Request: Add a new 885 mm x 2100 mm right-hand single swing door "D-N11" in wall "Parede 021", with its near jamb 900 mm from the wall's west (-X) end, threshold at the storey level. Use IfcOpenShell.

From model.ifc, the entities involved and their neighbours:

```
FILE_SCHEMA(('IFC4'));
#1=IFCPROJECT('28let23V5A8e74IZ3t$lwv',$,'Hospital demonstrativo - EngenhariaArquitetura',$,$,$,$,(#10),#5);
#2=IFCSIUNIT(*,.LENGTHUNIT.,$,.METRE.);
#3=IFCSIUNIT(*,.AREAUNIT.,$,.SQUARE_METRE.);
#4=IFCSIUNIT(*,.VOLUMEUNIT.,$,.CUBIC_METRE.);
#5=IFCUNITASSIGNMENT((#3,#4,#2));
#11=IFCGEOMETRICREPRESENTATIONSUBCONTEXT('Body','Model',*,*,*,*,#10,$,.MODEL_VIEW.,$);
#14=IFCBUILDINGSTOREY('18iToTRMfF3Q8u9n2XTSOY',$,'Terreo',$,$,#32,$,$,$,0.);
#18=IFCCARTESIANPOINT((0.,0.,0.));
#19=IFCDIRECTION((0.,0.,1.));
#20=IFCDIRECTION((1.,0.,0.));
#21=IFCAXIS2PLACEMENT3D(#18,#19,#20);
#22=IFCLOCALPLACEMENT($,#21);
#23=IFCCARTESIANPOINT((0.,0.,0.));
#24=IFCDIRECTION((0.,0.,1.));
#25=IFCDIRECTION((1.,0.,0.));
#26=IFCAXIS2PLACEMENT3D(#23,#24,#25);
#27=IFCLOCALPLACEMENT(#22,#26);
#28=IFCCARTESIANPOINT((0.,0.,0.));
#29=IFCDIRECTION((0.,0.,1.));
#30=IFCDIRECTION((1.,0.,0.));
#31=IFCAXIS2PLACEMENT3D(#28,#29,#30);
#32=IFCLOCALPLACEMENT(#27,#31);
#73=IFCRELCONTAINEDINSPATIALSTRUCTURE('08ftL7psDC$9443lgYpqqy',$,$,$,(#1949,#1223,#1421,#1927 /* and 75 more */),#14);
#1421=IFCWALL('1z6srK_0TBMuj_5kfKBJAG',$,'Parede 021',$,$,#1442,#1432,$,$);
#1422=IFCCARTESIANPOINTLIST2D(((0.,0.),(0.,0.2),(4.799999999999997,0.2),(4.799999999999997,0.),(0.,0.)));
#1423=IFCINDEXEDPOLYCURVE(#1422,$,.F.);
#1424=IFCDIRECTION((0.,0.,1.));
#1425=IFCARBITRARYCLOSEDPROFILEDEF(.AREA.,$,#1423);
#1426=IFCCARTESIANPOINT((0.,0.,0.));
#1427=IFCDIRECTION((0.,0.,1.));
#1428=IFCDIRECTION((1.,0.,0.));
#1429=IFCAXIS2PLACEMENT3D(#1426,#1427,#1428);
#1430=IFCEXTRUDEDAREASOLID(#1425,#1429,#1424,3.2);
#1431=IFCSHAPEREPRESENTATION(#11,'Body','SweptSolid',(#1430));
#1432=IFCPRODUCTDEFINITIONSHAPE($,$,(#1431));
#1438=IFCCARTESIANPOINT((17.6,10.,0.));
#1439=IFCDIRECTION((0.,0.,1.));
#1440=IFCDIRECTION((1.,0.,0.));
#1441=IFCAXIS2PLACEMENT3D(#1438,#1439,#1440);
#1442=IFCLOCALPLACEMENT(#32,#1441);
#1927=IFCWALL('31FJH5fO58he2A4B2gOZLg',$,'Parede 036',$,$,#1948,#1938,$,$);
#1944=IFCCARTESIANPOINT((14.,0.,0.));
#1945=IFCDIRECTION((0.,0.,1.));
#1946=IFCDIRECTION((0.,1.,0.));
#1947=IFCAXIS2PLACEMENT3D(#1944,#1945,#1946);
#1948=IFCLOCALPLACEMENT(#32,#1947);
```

```python
import numpy as np
import ifcopenshell
import ifcopenshell.api.feature
import ifcopenshell.api.geometry
import ifcopenshell.api.root
import ifcopenshell.api.spatial
import ifcopenshell.geom
import ifcopenshell.util.element
import ifcopenshell.util.placement
import ifcopenshell.util.representation
import ifcopenshell.util.shape
import ifcopenshell.util.unit

model = ifcopenshell.open("model.ifc")
unit_scale = ifcopenshell.util.unit.calculate_unit_scale(model)
settings = ifcopenshell.geom.settings()


def volume(element):
    """Net volume in cubic metres, openings subtracted."""
    shape = ifcopenshell.geom.create_shape(settings, element)
    return ifcopenshell.util.shape.get_volume(shape.geometry)


wall = model.by_guid("1z6srK_0TBMuj_5kfKBJAG")
storey = ifcopenshell.util.element.get_container(wall, ifc_class="IfcBuildingStorey")
context = ifcopenshell.util.representation.get_context(model, "Model", "Body", "MODEL_VIEW")
before = volume(wall)

width, height, from_end, sill = 0.885, 2.1, 0.9, 0.0  # metres

# The wall runs along its own X axis, and the end named is its -X end.
wall_shape = ifcopenshell.geom.create_shape(settings, wall)
x, y, z = ifcopenshell.util.shape.get_vertices(wall_shape.geometry).T
start = x.min() + from_end
face, thickness = float(y.min()), float(y.max() - y.min())
wall_matrix = ifcopenshell.util.placement.get_local_placement(wall.ObjectPlacement)
level = ifcopenshell.util.placement.get_local_placement(storey.ObjectPlacement)[2, 3]


def in_wall(x, y):
    """Placement at x, y metres in the wall's axes, at sill height."""
    matrix = wall_matrix.copy()
    matrix[:, 3] = wall_matrix @ np.array([x / unit_scale, y / unit_scale, 0.0, 1.0])
    matrix[2, 3] = level + sill / unit_scale
    return matrix


# Opening: a box that overshoots both wall faces by 50 mm.
opening = ifcopenshell.api.root.create_entity(model, ifc_class="IfcOpeningElement", predefined_type="OPENING")
box = ifcopenshell.api.geometry.add_wall_representation(
    model, context=context, length=width, height=height, thickness=thickness + 0.1
)
ifcopenshell.api.geometry.assign_representation(model, product=opening, representation=box)
ifcopenshell.api.geometry.edit_object_placement(model, product=opening, matrix=in_wall(start, face - 0.05), is_si=False)
ifcopenshell.api.feature.add_feature(model, feature=opening, element=wall)

door = ifcopenshell.api.root.create_entity(model, ifc_class="IfcDoor", name="D-N11", predefined_type="DOOR")
door.OverallWidth, door.OverallHeight = width / unit_scale, height / unit_scale
door.OperationType = "SINGLE_SWING_RIGHT"
body = ifcopenshell.api.geometry.add_door_representation(
    model,
    context=context,
    overall_width=door.OverallWidth,
    overall_height=door.OverallHeight,
    operation_type="SINGLE_SWING_RIGHT",
    lining_properties={"LiningDepth": thickness / unit_scale, "ThresholdDepth": thickness / unit_scale},
)
ifcopenshell.api.geometry.assign_representation(model, product=door, representation=body)
ifcopenshell.api.spatial.assign_container(model, products=[door], relating_structure=storey)
ifcopenshell.api.feature.add_filling(model, opening=opening, element=door)

# The lining spans the wall, so the door starts at the wall face.
ifcopenshell.api.geometry.edit_object_placement(model, product=door, matrix=in_wall(start, face), is_si=False)

after = volume(wall)

print(f"wall volume {before:.3f} -> {after:.3f} m3")

model.write("model_v2.ifc")
```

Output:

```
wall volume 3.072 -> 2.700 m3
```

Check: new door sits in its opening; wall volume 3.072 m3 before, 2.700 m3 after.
